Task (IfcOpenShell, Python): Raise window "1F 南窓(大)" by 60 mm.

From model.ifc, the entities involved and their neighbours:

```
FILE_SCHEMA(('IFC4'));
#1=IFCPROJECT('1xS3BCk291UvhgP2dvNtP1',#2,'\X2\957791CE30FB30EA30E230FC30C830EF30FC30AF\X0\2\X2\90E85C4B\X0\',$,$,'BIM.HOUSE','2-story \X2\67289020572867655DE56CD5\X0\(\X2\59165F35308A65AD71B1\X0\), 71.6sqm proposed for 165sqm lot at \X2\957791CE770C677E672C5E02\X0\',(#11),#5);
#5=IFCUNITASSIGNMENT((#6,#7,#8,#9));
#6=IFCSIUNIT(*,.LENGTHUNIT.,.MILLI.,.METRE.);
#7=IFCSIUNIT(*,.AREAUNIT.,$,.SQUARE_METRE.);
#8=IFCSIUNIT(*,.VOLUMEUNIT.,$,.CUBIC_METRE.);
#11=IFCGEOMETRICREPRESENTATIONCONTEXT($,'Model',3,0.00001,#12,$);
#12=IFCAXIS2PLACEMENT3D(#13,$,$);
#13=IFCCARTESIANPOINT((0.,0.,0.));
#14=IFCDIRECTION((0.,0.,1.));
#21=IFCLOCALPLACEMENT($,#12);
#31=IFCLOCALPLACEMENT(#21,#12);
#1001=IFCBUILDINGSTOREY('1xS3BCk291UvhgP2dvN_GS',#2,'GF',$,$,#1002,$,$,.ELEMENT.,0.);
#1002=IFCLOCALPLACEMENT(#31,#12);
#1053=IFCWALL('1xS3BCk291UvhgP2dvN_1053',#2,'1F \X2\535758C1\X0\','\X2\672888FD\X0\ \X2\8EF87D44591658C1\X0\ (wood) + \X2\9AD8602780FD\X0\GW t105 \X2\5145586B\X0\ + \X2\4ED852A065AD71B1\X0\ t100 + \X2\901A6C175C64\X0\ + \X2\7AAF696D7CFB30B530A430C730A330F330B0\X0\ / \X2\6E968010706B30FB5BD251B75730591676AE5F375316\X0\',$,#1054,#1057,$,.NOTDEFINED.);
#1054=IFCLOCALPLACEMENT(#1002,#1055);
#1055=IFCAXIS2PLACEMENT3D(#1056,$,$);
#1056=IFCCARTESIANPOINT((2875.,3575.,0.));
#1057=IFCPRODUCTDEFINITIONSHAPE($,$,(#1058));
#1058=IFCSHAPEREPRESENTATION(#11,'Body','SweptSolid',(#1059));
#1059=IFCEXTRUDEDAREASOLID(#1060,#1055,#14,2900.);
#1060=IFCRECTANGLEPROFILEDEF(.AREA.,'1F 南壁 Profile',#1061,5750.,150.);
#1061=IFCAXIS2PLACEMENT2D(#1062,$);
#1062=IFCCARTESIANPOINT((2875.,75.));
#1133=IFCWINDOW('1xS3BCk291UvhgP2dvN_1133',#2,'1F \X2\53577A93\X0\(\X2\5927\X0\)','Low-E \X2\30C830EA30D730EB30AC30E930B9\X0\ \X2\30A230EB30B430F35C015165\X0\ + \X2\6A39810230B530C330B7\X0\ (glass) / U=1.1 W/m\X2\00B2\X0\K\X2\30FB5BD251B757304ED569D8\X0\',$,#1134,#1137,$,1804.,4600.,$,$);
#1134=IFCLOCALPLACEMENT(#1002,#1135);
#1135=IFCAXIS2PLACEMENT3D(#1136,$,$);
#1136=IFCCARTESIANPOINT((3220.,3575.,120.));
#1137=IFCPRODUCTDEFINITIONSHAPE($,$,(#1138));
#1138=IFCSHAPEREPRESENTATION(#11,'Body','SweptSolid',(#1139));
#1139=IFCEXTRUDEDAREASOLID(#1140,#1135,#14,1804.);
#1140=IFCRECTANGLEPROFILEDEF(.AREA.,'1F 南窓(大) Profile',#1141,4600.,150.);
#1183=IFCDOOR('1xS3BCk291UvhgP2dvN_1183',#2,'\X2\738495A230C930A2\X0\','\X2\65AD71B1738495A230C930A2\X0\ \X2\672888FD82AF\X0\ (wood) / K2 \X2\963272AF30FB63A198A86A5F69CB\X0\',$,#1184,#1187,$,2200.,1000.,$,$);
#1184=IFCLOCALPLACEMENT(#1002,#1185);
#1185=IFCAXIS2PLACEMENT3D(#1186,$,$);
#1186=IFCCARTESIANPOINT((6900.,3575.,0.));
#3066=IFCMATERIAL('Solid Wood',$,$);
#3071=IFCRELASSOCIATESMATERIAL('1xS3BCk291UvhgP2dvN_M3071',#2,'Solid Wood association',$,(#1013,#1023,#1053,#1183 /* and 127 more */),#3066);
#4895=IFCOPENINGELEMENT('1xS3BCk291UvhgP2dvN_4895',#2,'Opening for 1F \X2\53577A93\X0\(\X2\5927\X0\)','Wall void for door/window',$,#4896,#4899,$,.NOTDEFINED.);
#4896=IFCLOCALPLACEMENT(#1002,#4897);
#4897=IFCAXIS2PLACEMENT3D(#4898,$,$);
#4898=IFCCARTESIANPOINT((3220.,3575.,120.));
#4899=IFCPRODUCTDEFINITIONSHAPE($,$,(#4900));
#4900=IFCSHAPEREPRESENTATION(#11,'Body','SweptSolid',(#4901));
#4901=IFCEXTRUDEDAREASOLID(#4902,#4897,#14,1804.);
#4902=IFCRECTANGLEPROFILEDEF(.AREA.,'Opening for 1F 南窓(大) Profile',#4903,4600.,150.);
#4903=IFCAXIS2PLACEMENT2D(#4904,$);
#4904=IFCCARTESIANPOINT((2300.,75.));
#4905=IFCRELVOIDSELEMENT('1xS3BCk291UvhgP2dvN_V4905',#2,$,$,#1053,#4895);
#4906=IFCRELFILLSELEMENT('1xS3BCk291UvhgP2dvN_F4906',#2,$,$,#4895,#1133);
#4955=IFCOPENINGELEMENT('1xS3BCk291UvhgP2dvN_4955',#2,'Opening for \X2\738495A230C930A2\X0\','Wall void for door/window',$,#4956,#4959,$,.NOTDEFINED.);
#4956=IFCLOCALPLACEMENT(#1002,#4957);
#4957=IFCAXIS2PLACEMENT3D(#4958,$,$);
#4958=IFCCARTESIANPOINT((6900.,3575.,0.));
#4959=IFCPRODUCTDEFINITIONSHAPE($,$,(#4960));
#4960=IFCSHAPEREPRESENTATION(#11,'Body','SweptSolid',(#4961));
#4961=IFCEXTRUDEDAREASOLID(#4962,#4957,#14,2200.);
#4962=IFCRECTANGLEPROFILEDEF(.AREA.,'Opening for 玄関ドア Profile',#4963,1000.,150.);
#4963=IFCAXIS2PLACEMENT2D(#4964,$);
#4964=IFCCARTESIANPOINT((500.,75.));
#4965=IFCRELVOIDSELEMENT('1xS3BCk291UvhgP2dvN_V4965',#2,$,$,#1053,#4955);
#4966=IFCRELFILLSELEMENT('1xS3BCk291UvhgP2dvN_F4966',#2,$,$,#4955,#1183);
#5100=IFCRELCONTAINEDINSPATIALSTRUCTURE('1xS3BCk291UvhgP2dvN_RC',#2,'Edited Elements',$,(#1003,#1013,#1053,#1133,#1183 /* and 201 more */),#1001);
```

```python
import numpy as np
import ifcopenshell
import ifcopenshell.api.geometry
import ifcopenshell.util.placement
import ifcopenshell.util.unit

model = ifcopenshell.open("model.ifc")
unit_scale = ifcopenshell.util.unit.calculate_unit_scale(model)

window = model.by_guid("1xS3BCk291UvhgP2dvN_1133")
opening = window.FillsVoids[0].RelatingOpeningElement
dz = 0.06 / unit_scale

shift = np.array([0.0, 0.0, dz])
# The window is not placed relative to its opening, so move both.
for product in (opening, window):
    matrix = ifcopenshell.util.placement.get_local_placement(product.ObjectPlacement)
    matrix[:3, 3] += shift
    ifcopenshell.api.geometry.edit_object_placement(model, product=product, matrix=matrix, is_si=False)

print(f"moved by {dz * unit_scale:+.3f} m")

model.write("model_rev.ifc")
```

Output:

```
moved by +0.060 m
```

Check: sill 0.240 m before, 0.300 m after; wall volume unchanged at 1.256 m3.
